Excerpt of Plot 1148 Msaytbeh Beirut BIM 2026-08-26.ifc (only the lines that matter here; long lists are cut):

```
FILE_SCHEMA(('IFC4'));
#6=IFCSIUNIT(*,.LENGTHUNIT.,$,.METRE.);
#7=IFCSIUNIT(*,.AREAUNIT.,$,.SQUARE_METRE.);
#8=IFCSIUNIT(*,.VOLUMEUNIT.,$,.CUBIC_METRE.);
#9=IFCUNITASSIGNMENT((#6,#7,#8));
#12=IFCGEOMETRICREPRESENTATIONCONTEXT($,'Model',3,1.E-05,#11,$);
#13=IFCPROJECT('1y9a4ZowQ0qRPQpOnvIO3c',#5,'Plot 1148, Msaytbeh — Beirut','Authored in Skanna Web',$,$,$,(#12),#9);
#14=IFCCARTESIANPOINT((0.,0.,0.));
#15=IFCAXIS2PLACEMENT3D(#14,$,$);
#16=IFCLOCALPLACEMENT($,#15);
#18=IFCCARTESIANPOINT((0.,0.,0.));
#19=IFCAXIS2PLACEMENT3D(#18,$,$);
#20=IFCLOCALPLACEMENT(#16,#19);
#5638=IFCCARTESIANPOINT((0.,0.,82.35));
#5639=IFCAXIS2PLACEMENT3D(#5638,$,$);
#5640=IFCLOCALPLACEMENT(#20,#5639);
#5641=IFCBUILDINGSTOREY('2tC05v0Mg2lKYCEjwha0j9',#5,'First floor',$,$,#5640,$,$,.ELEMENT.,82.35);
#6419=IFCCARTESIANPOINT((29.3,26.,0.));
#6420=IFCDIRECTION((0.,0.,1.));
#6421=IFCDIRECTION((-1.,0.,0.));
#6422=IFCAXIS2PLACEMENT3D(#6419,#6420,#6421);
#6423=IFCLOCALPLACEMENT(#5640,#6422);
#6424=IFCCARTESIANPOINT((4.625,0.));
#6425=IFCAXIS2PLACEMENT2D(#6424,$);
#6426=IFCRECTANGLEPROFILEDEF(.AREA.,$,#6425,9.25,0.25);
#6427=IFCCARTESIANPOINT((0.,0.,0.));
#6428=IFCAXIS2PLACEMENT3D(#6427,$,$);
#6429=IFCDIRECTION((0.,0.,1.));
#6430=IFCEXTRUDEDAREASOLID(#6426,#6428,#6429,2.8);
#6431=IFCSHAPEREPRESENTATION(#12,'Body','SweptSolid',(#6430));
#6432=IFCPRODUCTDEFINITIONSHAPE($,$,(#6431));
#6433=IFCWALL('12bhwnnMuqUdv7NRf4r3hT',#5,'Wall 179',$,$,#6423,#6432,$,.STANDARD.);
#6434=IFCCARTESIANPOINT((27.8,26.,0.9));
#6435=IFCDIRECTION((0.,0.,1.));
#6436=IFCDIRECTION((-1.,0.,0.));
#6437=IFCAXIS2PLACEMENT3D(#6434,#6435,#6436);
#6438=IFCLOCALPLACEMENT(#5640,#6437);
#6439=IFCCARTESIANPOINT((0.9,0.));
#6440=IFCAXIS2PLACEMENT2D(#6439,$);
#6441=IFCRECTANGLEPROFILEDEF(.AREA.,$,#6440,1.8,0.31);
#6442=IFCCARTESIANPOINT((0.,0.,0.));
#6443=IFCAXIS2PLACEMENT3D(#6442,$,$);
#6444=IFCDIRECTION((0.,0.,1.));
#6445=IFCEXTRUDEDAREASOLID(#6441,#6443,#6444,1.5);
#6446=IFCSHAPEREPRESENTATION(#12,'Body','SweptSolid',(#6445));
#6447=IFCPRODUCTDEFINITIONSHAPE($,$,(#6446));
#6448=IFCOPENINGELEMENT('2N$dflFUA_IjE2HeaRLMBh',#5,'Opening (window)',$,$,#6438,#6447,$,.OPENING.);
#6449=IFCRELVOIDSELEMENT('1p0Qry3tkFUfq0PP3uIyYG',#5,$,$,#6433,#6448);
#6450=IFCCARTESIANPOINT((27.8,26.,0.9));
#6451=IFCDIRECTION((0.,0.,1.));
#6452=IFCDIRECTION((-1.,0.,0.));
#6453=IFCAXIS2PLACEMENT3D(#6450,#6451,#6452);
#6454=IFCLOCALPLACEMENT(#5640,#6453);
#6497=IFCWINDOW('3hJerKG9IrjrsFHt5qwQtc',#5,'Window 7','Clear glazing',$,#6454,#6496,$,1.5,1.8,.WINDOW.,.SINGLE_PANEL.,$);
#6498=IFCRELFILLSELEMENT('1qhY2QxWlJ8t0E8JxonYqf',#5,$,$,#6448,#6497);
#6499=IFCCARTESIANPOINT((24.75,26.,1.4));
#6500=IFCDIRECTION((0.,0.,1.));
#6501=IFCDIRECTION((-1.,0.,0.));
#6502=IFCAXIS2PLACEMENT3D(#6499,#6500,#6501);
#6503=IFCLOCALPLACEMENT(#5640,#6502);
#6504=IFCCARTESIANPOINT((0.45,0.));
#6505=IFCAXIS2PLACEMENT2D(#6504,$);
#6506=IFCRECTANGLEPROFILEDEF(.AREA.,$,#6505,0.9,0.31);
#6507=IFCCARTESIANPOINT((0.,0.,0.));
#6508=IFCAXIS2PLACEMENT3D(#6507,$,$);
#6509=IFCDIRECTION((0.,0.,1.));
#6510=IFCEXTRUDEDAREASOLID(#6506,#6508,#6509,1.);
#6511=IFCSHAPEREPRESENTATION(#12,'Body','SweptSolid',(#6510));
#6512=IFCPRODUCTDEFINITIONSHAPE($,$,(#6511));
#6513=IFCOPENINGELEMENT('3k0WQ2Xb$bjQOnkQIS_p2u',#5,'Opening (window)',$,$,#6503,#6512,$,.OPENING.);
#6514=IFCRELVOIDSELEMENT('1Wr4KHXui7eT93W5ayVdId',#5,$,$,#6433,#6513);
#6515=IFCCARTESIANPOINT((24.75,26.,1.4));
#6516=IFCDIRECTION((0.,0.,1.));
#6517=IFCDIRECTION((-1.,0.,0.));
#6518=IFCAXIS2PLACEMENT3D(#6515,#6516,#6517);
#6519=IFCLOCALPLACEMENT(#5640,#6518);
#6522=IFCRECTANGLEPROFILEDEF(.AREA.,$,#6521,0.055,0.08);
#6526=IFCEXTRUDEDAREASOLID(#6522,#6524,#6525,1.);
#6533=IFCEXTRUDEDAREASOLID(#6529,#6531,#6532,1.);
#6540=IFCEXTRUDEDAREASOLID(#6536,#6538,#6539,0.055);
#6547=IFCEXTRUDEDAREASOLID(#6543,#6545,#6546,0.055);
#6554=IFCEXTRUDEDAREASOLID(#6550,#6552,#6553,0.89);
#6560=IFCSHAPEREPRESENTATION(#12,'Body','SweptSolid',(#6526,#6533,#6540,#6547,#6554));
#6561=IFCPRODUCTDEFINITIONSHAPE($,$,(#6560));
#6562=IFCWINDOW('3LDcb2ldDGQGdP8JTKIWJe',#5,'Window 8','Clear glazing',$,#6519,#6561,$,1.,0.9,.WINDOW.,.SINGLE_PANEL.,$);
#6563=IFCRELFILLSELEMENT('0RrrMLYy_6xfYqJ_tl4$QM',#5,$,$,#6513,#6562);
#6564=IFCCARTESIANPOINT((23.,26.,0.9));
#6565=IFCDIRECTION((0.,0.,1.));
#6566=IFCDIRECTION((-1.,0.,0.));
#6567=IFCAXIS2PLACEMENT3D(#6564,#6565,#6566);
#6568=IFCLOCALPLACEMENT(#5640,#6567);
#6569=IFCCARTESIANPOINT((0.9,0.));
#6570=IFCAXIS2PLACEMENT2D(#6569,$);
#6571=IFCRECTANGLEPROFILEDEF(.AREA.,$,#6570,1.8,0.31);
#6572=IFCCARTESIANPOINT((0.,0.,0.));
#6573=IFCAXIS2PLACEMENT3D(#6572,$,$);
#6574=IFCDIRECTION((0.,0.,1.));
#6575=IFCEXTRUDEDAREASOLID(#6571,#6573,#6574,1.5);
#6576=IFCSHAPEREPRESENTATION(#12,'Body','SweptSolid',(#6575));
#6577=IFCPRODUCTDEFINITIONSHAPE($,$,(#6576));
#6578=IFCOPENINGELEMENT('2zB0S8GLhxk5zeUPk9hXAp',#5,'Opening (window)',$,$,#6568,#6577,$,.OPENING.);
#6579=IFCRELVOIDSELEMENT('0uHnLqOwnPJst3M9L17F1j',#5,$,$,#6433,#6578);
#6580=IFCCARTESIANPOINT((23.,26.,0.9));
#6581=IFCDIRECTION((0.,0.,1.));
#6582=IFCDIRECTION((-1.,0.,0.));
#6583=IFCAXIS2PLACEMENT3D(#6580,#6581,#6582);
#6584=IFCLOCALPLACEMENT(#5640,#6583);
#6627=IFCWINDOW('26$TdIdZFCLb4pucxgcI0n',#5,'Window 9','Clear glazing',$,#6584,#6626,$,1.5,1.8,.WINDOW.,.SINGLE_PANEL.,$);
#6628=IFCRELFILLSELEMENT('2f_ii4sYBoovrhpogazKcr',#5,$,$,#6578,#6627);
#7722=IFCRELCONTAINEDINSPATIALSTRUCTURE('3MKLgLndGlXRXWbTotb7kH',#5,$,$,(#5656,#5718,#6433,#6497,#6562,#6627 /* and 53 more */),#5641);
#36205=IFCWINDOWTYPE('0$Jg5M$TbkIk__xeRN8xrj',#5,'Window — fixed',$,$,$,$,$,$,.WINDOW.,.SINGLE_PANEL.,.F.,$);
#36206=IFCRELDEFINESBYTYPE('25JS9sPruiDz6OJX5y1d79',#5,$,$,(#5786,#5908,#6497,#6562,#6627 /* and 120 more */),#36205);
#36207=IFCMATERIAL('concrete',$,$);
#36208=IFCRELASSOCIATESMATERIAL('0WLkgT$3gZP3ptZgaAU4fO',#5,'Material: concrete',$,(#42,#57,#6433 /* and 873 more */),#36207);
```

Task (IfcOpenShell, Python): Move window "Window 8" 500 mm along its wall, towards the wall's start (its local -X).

```python
import ifcopenshell
import ifcopenshell.api.geometry
import ifcopenshell.util.placement
import ifcopenshell.util.unit

model = ifcopenshell.open("Plot 1148 Msaytbeh Beirut BIM 2026-08-26.ifc")
unit_scale = ifcopenshell.util.unit.calculate_unit_scale(model)

window = model.by_guid("3LDcb2ldDGQGdP8JTKIWJe")
opening = window.FillsVoids[0].RelatingOpeningElement
wall = opening.VoidsElements[0].RelatingBuildingElement

wall_matrix = ifcopenshell.util.placement.get_local_placement(wall.ObjectPlacement)
shift = wall_matrix[:3, 0] * -0.5 / unit_scale
before = ifcopenshell.util.placement.get_local_placement(window.ObjectPlacement)[:3, 3].copy()

# The window is not placed relative to its opening, so move both.
for product in (opening, window):
    matrix = ifcopenshell.util.placement.get_local_placement(product.ObjectPlacement)
    matrix[:3, 3] += shift
    ifcopenshell.api.geometry.edit_object_placement(model, product=product, matrix=matrix, is_si=False)

after = ifcopenshell.util.placement.get_local_placement(window.ObjectPlacement)[:3, 3]
print("window moved by", (after - before).round(3) + 0.0)

model.write("Plot 1148 Msaytbeh Beirut BIM 2026-08-26_v2.ifc")
```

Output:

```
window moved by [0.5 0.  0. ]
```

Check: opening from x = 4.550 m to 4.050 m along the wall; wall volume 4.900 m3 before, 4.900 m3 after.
